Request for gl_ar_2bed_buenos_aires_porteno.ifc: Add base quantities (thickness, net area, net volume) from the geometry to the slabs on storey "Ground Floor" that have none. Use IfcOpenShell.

First a look at what the model holds.

```python
import ifcopenshell
import ifcopenshell.util.element
import ifcopenshell.util.unit

model = ifcopenshell.open("gl_ar_2bed_buenos_aires_porteno.ifc")
print(model.schema)
for unit_type in ("LENGTHUNIT", "AREAUNIT", "VOLUMEUNIT"):
    print(unit_type, ifcopenshell.util.unit.calculate_unit_scale(model, unit_type))
storey = next(s for s in model.by_type("IfcBuildingStorey") if s.Name == "Ground Floor")
slabs = [e for e in ifcopenshell.util.element.get_decomposition(storey) if e.is_a("IfcSlab")]
for e in sorted(slabs, key=lambda e: e.id()):
    print(e.id(), e.is_a(), e.Name, list(ifcopenshell.util.element.get_psets(e, qtos_only=True)), sep=" | ")
```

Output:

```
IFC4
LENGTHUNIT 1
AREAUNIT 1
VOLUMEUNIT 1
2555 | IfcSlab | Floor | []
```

```python
import ifcopenshell
import ifcopenshell.api.pset
import ifcopenshell.geom
import ifcopenshell.util.element
import ifcopenshell.util.shape
import ifcopenshell.util.unit

model = ifcopenshell.open("gl_ar_2bed_buenos_aires_porteno.ifc")
unit_scale = ifcopenshell.util.unit.calculate_unit_scale(model)
area_scale = ifcopenshell.util.unit.calculate_unit_scale(model, "AREAUNIT")
volume_scale = ifcopenshell.util.unit.calculate_unit_scale(model, "VOLUMEUNIT")
settings = ifcopenshell.geom.settings()

storey = next(s for s in model.by_type("IfcBuildingStorey") if s.Name == "Ground Floor")
slabs = [e for e in ifcopenshell.util.element.get_decomposition(storey) if e.is_a("IfcSlab")]

for e in sorted(slabs, key=lambda e: e.id()):
    if ifcopenshell.util.element.get_psets(e, qtos_only=True, should_inherit=False):
        continue
    # Geometry comes back in metres, in the element's own axes.
    shape = ifcopenshell.geom.create_shape(settings, e)
    values = {
        "Width": ifcopenshell.util.shape.get_z(shape.geometry) / unit_scale,
        "NetArea": ifcopenshell.util.shape.get_footprint_area(shape.geometry) / area_scale,
        "NetVolume": ifcopenshell.util.shape.get_volume(shape.geometry) / volume_scale,
    }
    qto = ifcopenshell.api.pset.add_qto(model, product=e, name="Qto_SlabBaseQuantities")
    ifcopenshell.api.pset.edit_qto(model, qto=qto, properties=values)
    print(e.id(), {k: round(v, 3) for k, v in values.items()})

model.write("gl_ar_2bed_buenos_aires_porteno_updated.ifc")
```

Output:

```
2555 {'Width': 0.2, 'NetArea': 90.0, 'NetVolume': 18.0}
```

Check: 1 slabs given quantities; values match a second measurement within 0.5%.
